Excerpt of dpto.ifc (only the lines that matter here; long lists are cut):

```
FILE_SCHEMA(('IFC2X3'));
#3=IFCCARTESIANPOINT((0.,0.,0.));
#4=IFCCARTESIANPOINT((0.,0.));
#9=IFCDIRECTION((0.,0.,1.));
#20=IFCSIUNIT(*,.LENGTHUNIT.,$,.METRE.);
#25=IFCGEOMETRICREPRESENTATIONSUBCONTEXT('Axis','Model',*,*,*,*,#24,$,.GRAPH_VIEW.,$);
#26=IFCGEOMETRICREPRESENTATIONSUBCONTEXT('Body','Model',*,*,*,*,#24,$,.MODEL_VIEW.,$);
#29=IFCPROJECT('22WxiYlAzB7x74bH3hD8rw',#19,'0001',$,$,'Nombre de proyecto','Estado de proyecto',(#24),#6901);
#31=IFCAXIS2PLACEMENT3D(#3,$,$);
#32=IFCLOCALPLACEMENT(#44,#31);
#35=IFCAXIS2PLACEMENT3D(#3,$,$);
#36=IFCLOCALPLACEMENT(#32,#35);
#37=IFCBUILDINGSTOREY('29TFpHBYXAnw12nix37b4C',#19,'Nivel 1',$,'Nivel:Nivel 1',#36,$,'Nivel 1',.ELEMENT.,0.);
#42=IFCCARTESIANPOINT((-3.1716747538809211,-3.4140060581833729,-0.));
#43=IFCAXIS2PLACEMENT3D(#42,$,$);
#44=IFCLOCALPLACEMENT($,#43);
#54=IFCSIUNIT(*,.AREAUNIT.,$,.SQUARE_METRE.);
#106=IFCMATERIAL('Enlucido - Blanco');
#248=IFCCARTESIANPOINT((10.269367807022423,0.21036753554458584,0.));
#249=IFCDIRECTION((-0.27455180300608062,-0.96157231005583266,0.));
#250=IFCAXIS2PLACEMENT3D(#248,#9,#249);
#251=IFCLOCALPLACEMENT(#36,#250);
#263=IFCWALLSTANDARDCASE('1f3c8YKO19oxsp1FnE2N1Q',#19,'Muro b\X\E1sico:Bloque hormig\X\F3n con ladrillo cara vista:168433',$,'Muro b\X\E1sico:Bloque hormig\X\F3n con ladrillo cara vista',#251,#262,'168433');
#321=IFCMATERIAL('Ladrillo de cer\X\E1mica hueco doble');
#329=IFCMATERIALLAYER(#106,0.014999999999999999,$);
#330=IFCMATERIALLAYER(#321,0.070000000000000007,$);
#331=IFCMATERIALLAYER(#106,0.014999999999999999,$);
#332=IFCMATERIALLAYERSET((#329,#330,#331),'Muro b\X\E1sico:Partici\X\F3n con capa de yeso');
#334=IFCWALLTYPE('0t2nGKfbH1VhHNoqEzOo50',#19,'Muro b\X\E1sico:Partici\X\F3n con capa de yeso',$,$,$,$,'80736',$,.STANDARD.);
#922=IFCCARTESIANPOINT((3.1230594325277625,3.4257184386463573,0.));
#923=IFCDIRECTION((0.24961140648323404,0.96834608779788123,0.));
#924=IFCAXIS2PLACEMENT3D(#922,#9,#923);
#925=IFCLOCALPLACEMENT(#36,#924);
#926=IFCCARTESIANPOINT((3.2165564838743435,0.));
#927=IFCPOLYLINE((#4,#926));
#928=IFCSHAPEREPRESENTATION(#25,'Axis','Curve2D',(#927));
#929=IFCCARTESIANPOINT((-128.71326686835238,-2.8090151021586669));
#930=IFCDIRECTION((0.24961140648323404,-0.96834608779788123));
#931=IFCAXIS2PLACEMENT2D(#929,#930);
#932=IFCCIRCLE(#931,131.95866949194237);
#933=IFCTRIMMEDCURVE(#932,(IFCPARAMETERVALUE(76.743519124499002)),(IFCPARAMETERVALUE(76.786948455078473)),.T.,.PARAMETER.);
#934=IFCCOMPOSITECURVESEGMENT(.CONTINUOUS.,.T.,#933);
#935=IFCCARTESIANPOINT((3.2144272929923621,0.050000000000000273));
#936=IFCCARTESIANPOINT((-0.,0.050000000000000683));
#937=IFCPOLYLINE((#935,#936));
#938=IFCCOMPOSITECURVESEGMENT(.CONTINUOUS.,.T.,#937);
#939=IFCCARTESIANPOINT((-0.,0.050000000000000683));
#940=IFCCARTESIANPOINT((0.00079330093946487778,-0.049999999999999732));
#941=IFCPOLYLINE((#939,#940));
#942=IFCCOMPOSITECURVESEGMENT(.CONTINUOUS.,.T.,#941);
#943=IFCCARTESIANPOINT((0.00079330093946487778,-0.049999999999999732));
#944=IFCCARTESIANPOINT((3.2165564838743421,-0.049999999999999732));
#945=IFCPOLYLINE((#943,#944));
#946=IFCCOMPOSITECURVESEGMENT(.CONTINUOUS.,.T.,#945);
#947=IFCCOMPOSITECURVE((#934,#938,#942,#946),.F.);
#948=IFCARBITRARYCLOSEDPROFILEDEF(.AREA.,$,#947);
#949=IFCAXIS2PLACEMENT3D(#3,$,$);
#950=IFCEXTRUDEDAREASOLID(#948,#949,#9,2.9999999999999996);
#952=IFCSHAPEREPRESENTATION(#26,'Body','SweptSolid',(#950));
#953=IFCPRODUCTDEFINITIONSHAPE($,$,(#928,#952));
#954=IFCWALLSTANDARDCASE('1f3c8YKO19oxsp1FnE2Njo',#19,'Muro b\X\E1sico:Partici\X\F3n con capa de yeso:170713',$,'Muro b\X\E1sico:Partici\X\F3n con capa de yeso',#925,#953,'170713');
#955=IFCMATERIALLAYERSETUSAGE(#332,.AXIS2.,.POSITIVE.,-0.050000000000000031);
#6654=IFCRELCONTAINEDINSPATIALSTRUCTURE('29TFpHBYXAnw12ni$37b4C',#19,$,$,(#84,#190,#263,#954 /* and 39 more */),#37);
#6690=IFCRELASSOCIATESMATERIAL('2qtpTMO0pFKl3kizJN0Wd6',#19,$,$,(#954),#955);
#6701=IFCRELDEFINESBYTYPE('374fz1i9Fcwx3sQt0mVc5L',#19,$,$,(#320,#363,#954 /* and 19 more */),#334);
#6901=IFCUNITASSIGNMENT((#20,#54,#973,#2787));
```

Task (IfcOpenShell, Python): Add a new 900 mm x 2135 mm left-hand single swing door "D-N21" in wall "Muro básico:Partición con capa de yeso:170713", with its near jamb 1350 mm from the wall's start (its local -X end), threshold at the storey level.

```python
import numpy as np
import ifcopenshell
import ifcopenshell.api.feature
import ifcopenshell.api.geometry
import ifcopenshell.api.root
import ifcopenshell.api.spatial
import ifcopenshell.api.type
import ifcopenshell.geom
import ifcopenshell.util.element
import ifcopenshell.util.placement
import ifcopenshell.util.representation
import ifcopenshell.util.shape
import ifcopenshell.util.unit

model = ifcopenshell.open("dpto.ifc")
unit_scale = ifcopenshell.util.unit.calculate_unit_scale(model)
settings = ifcopenshell.geom.settings()


def volume(element):
    """Net volume in cubic metres, openings subtracted."""
    shape = ifcopenshell.geom.create_shape(settings, element)
    return ifcopenshell.util.shape.get_volume(shape.geometry)


wall = model.by_guid("1f3c8YKO19oxsp1FnE2Njo")
storey = ifcopenshell.util.element.get_container(wall, ifc_class="IfcBuildingStorey")
context = ifcopenshell.util.representation.get_context(model, "Model", "Body", "MODEL_VIEW")
before = volume(wall)

width, height, from_end, sill = 0.9, 2.135, 1.35, 0.0  # metres

# The wall runs along its own X axis, and the end named is its -X end.
wall_shape = ifcopenshell.geom.create_shape(settings, wall)
x, y, z = ifcopenshell.util.shape.get_vertices(wall_shape.geometry).T
start = x.min() + from_end
face, thickness = float(y.min()), float(y.max() - y.min())
wall_matrix = ifcopenshell.util.placement.get_local_placement(wall.ObjectPlacement)
level = ifcopenshell.util.placement.get_local_placement(storey.ObjectPlacement)[2, 3]


def in_wall(x, y):
    """Placement at x, y metres in the wall's axes, at sill height."""
    matrix = wall_matrix.copy()
    matrix[:, 3] = wall_matrix @ np.array([x / unit_scale, y / unit_scale, 0.0, 1.0])
    matrix[2, 3] = level + sill / unit_scale
    return matrix


# Opening: a box that overshoots both wall faces by 50 mm.
opening = ifcopenshell.api.root.create_entity(model, ifc_class="IfcOpeningElement")
box = ifcopenshell.api.geometry.add_wall_representation(
    model, context=context, length=width, height=height, thickness=thickness + 0.1
)
ifcopenshell.api.geometry.assign_representation(model, product=opening, representation=box)
ifcopenshell.api.geometry.edit_object_placement(model, product=opening, matrix=in_wall(start, face - 0.05), is_si=False)
ifcopenshell.api.feature.add_feature(model, feature=opening, element=wall)

door = ifcopenshell.api.root.create_entity(model, ifc_class="IfcDoor", name="D-N21")
door.OverallWidth, door.OverallHeight = width / unit_scale, height / unit_scale
body = ifcopenshell.api.geometry.add_door_representation(
    model,
    context=context,
    overall_width=door.OverallWidth,
    overall_height=door.OverallHeight,
    operation_type="SINGLE_SWING_LEFT",
    lining_properties={"LiningDepth": thickness / unit_scale, "ThresholdDepth": thickness / unit_scale},
)
ifcopenshell.api.geometry.assign_representation(model, product=door, representation=body)
ifcopenshell.api.spatial.assign_container(model, products=[door], relating_structure=storey)
fills = ifcopenshell.api.feature.add_filling(model, opening=opening, element=door)
fills.OwnerHistory = door.OwnerHistory  # required in IFC2X3

# IFC2X3 keeps the operation on the door style.
style = ifcopenshell.api.root.create_entity(model, ifc_class="IfcDoorStyle", name="D-N21")
style.OperationType, style.ConstructionType = "SINGLE_SWING_LEFT", "NOTDEFINED"
style.ParameterTakesPrecedence = style.Sizeable = False
ifcopenshell.api.type.assign_type(model, related_objects=[door], relating_type=style)

# The lining spans the wall, so the door starts at the wall face.
ifcopenshell.api.geometry.edit_object_placement(model, product=door, matrix=in_wall(start, face), is_si=False)

after = volume(wall)

print(f"wall volume {before:.3f} -> {after:.3f} m3")

model.write("dpto-out.ifc")
```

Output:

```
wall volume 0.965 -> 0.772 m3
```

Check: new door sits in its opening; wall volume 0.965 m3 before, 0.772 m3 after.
